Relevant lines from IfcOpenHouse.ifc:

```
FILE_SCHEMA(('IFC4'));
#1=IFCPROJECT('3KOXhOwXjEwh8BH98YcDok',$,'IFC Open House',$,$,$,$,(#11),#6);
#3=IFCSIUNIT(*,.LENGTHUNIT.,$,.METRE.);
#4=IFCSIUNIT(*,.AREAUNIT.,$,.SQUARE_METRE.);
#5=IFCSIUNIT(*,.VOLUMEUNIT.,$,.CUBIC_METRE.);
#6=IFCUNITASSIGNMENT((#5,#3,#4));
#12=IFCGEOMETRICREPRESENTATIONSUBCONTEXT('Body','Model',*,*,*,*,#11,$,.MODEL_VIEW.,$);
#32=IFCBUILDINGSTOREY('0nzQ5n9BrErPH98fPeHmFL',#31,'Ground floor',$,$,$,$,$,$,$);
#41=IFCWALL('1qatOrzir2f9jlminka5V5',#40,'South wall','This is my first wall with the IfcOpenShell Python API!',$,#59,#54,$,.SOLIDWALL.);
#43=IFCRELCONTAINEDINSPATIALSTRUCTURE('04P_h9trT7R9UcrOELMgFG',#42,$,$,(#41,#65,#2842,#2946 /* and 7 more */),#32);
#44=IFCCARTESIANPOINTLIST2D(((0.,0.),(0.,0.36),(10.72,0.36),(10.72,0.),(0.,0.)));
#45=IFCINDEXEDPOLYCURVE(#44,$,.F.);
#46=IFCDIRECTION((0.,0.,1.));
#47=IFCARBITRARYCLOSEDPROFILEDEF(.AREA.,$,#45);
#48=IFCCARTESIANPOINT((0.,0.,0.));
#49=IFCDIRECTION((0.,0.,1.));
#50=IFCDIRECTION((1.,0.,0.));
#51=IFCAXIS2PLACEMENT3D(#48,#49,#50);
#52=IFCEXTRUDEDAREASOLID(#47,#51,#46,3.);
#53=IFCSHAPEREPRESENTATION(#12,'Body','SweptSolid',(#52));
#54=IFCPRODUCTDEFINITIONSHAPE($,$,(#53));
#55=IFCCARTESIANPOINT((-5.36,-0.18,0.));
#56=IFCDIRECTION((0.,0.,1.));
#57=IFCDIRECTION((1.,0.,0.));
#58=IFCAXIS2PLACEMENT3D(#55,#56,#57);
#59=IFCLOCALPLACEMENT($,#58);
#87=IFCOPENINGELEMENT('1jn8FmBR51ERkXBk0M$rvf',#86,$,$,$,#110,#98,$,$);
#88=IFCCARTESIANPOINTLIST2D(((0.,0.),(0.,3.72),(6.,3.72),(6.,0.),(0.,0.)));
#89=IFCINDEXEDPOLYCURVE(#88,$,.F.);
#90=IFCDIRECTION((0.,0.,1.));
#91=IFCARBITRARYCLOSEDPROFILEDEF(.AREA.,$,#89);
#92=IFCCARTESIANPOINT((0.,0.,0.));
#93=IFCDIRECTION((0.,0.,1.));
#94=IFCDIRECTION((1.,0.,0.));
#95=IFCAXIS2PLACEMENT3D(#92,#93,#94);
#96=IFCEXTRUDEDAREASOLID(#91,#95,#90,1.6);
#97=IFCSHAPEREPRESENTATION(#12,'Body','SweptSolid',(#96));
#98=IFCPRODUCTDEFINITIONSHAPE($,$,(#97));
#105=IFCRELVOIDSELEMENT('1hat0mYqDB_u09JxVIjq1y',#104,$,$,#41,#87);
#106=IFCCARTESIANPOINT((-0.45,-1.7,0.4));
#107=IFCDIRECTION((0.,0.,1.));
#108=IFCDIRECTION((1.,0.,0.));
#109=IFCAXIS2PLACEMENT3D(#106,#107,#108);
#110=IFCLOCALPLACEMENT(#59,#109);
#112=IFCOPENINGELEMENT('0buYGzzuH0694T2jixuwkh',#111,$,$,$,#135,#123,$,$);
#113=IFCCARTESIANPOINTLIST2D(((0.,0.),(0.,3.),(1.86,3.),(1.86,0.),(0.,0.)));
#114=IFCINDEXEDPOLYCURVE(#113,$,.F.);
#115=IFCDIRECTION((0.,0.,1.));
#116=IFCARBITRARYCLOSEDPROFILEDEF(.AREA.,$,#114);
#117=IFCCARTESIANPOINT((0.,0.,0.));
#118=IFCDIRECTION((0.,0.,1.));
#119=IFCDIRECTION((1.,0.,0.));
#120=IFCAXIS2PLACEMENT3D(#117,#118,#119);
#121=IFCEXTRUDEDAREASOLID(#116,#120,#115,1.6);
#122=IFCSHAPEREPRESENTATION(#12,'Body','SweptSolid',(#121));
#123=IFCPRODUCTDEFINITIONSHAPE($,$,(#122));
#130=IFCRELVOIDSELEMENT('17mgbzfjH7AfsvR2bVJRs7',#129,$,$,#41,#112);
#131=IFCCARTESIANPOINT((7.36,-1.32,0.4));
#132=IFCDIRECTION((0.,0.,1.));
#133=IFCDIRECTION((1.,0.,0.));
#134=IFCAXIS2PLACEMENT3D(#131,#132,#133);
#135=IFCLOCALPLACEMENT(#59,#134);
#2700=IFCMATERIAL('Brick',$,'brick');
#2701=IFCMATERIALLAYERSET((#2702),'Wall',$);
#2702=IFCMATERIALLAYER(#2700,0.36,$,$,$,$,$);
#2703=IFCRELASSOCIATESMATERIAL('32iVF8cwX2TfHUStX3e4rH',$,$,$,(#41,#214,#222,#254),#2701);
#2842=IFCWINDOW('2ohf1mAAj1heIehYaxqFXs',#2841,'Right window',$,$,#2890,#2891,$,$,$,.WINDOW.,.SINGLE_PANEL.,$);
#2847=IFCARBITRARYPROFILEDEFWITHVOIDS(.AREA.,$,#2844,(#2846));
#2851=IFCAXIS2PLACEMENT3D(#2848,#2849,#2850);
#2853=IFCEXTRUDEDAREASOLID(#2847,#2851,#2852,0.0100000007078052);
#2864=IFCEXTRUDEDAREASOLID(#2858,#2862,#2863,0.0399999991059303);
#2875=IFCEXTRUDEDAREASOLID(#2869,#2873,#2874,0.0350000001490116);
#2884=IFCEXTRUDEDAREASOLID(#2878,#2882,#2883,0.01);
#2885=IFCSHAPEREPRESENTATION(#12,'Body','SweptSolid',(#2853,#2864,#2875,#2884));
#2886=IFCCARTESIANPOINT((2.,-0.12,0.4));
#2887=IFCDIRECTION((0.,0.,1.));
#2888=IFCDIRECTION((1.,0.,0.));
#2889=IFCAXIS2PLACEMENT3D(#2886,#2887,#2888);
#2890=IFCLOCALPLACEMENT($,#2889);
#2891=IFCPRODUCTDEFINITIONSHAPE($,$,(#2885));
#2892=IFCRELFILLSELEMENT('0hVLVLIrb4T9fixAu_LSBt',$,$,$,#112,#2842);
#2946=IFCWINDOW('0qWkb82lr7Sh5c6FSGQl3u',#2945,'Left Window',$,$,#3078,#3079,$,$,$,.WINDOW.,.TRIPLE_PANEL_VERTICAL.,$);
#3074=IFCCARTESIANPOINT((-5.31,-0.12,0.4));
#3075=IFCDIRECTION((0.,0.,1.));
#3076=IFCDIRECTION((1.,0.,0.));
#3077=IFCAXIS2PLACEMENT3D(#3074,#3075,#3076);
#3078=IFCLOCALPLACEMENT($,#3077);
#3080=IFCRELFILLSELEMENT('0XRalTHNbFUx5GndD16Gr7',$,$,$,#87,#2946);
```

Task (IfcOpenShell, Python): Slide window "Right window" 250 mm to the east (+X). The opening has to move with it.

```python
import ifcopenshell
import ifcopenshell.api.geometry
import ifcopenshell.util.placement

model = ifcopenshell.open("IfcOpenHouse.ifc")

window = model.by_guid("2ohf1mAAj1heIehYaxqFXs")
opening = window.FillsVoids[0].RelatingOpeningElement
wall = opening.VoidsElements[0].RelatingBuildingElement

wall_matrix = ifcopenshell.util.placement.get_local_placement(wall.ObjectPlacement)
shift = wall_matrix[:3, 0] * 0.25
before = ifcopenshell.util.placement.get_local_placement(window.ObjectPlacement)[:3, 3].copy()

# The window is not placed relative to its opening, so move both.
for product in (opening, window):
    matrix = ifcopenshell.util.placement.get_local_placement(product.ObjectPlacement)
    matrix[:3, 3] += shift
    ifcopenshell.api.geometry.edit_object_placement(model, product=product, matrix=matrix, is_si=False)

after = ifcopenshell.util.placement.get_local_placement(window.ObjectPlacement)[:3, 3]
print("window moved by", (after - before).round(3) + 0.0)

model.write("IfcOpenHouse_updated.ifc")
```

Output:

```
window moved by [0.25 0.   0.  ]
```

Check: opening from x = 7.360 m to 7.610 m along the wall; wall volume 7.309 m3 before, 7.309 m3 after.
